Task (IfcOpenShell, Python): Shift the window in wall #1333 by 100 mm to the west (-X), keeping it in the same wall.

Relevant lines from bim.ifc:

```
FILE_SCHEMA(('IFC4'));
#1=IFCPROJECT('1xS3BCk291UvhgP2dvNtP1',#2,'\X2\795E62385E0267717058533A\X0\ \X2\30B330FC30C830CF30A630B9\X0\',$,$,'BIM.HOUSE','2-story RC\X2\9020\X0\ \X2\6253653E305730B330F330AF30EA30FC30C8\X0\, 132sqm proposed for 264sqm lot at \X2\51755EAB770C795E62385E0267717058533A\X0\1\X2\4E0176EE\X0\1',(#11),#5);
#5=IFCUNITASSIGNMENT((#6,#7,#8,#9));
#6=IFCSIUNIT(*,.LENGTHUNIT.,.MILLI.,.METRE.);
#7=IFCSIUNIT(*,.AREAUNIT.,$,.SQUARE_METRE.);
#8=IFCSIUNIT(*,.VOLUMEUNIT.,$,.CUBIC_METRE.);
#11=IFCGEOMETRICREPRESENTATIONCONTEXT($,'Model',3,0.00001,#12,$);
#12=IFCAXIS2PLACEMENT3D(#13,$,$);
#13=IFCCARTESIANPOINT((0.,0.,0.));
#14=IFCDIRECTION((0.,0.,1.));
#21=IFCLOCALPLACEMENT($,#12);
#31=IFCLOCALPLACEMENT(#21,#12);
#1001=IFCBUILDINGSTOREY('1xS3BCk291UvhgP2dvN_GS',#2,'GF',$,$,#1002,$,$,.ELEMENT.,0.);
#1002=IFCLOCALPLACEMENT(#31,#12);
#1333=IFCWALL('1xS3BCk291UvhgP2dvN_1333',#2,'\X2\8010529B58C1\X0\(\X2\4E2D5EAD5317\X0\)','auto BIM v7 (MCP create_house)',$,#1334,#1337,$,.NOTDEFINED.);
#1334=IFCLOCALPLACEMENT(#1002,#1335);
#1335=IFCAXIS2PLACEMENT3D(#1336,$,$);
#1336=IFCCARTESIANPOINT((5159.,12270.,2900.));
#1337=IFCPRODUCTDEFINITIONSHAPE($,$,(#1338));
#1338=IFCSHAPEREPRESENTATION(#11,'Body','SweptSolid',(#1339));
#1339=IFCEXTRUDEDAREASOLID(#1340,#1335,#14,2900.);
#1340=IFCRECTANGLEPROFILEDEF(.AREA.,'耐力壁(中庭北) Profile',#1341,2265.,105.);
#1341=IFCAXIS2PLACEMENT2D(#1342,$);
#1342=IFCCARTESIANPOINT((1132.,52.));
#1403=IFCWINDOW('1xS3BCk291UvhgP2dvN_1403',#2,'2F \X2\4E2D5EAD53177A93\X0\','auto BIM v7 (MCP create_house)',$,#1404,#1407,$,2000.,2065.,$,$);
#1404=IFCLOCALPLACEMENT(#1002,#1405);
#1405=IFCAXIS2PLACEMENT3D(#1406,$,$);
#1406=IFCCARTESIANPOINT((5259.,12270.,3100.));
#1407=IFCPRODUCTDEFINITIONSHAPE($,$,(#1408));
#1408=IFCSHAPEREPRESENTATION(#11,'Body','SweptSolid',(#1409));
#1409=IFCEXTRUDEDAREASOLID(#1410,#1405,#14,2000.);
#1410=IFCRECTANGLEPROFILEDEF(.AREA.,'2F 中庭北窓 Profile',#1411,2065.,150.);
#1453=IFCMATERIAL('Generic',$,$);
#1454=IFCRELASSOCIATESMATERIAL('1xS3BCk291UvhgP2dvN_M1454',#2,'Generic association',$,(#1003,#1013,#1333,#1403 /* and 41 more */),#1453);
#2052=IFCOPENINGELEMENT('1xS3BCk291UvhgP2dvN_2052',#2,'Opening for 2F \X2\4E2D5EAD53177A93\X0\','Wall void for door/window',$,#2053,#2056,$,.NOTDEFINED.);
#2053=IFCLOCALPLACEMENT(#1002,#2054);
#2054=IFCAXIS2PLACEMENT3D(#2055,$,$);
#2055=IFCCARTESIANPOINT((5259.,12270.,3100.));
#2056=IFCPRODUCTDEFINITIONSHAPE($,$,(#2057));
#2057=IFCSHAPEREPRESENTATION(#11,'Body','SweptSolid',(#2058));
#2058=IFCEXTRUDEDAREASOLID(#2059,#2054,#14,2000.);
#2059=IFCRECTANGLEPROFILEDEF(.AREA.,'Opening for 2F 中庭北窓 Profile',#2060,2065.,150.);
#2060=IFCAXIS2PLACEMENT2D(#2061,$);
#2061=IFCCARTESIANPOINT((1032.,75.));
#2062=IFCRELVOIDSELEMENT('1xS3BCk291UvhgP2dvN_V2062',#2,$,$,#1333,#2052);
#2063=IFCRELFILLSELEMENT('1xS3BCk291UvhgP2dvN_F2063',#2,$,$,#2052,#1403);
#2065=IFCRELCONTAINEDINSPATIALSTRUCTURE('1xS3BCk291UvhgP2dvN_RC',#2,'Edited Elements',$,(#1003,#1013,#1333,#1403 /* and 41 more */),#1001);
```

```python
import ifcopenshell
import ifcopenshell.api.geometry
import ifcopenshell.util.placement

model = ifcopenshell.open("bim.ifc")

window = model.by_id(1403)
opening = window.FillsVoids[0].RelatingOpeningElement
wall = opening.VoidsElements[0].RelatingBuildingElement

wall_matrix = ifcopenshell.util.placement.get_local_placement(wall.ObjectPlacement)
shift = wall_matrix[:3, 0] * -100.0
before = ifcopenshell.util.placement.get_local_placement(window.ObjectPlacement)[:3, 3].copy()

# The window is not placed relative to its opening, so move both.
for product in (opening, window):
    matrix = ifcopenshell.util.placement.get_local_placement(product.ObjectPlacement)
    matrix[:3, 3] += shift
    ifcopenshell.api.geometry.edit_object_placement(model, product=product, matrix=matrix, is_si=False)

after = ifcopenshell.util.placement.get_local_placement(window.ObjectPlacement)[:3, 3]
print("window moved by", (after - before).round(3) + 0.0)

model.write("bim_v2.ifc")
```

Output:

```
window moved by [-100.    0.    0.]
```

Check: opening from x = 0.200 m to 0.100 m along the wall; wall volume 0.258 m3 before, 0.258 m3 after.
